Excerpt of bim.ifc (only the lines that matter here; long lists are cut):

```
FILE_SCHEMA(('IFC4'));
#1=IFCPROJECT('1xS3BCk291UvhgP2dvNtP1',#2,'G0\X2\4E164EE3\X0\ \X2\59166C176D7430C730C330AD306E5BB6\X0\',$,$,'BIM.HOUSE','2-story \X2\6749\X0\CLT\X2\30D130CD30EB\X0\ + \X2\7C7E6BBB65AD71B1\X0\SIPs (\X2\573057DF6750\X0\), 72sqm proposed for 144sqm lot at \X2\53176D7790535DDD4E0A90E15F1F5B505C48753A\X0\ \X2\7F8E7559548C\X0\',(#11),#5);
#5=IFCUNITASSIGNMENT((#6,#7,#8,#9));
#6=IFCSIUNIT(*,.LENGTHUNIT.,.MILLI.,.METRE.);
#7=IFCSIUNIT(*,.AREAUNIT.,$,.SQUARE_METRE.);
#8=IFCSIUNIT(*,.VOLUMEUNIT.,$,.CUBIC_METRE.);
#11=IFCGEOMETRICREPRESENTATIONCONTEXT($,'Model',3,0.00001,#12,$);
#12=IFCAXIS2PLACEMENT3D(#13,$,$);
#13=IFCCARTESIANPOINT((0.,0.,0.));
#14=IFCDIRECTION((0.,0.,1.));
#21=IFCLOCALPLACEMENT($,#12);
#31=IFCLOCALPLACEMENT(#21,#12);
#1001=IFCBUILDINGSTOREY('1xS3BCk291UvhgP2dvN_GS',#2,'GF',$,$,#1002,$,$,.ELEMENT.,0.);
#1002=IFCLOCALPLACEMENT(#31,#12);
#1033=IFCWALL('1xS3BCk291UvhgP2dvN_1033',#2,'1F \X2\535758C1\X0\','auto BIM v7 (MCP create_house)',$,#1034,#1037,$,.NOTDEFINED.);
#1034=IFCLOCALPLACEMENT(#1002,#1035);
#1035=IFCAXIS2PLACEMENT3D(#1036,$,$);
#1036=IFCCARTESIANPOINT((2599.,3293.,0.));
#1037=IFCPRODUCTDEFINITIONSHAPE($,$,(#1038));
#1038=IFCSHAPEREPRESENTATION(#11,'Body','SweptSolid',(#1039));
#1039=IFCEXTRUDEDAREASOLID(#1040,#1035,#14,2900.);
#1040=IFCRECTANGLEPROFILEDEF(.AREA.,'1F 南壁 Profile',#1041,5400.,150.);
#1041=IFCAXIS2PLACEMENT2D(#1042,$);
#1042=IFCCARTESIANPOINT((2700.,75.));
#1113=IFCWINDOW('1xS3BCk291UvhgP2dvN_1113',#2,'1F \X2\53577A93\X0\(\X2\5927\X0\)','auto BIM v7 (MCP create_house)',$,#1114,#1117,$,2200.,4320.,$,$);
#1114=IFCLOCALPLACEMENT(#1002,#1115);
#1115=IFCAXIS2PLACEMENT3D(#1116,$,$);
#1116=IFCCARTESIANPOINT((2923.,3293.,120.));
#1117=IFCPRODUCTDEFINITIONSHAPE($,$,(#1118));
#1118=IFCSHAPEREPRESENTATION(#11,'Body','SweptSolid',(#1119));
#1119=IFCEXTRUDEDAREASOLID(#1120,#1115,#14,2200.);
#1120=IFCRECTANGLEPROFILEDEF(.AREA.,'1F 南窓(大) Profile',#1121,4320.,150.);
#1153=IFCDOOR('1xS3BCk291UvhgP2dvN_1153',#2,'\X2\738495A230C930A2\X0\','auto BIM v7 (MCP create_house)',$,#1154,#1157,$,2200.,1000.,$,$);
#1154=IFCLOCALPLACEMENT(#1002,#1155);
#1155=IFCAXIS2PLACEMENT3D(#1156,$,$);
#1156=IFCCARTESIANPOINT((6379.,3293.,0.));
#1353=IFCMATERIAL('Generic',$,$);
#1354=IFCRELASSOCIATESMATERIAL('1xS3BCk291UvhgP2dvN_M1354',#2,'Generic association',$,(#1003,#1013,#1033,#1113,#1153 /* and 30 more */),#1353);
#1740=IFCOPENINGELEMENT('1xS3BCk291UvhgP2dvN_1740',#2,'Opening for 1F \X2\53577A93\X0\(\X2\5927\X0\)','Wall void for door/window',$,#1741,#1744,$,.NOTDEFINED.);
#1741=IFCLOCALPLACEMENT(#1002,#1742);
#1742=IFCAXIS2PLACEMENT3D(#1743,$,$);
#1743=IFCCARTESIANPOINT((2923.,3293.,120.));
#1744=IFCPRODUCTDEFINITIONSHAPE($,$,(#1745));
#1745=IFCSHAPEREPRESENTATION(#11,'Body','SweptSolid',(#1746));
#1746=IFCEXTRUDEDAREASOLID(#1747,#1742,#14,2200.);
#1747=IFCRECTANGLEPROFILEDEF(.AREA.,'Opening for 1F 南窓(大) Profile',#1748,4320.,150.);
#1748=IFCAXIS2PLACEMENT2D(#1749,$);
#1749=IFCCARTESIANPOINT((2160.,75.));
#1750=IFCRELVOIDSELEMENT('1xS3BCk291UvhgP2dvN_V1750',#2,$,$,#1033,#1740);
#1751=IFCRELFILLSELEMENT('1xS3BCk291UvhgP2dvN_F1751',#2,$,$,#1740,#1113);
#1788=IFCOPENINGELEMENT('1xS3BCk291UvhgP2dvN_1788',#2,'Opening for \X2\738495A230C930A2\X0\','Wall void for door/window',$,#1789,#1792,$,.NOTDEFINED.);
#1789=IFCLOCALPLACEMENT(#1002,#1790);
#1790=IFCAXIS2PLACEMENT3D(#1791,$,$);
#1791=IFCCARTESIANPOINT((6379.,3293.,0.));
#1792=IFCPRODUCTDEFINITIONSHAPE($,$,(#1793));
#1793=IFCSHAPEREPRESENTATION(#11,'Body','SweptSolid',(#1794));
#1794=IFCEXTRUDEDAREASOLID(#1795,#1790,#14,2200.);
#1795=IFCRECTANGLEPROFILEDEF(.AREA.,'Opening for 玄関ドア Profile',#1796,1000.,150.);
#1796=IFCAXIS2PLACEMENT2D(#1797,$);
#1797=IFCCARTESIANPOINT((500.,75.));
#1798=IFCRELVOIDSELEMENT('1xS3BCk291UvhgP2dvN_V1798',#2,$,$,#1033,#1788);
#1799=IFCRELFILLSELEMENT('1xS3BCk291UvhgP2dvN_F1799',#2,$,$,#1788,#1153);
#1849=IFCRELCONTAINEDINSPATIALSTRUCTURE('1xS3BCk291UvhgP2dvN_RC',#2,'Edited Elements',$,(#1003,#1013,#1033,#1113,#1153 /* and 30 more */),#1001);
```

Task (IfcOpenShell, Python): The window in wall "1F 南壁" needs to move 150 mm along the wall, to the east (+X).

```python
import ifcopenshell
import ifcopenshell.api.geometry
import ifcopenshell.util.placement
import ifcopenshell.util.unit

model = ifcopenshell.open("bim.ifc")
unit_scale = ifcopenshell.util.unit.calculate_unit_scale(model)

window = model.by_id(1113)
opening = window.FillsVoids[0].RelatingOpeningElement
wall = opening.VoidsElements[0].RelatingBuildingElement

wall_matrix = ifcopenshell.util.placement.get_local_placement(wall.ObjectPlacement)
shift = wall_matrix[:3, 0] * 0.15 / unit_scale
before = ifcopenshell.util.placement.get_local_placement(window.ObjectPlacement)[:3, 3].copy()

# The window is not placed relative to its opening, so move both.
for product in (opening, window):
    matrix = ifcopenshell.util.placement.get_local_placement(product.ObjectPlacement)
    matrix[:3, 3] += shift
    ifcopenshell.api.geometry.edit_object_placement(model, product=product, matrix=matrix, is_si=False)

after = ifcopenshell.util.placement.get_local_placement(window.ObjectPlacement)[:3, 3]
print("window moved by", (after - before).round(3) + 0.0)

model.write("bim_updated.ifc")
```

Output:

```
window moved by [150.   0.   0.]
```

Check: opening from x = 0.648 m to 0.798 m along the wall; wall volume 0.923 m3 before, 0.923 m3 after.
